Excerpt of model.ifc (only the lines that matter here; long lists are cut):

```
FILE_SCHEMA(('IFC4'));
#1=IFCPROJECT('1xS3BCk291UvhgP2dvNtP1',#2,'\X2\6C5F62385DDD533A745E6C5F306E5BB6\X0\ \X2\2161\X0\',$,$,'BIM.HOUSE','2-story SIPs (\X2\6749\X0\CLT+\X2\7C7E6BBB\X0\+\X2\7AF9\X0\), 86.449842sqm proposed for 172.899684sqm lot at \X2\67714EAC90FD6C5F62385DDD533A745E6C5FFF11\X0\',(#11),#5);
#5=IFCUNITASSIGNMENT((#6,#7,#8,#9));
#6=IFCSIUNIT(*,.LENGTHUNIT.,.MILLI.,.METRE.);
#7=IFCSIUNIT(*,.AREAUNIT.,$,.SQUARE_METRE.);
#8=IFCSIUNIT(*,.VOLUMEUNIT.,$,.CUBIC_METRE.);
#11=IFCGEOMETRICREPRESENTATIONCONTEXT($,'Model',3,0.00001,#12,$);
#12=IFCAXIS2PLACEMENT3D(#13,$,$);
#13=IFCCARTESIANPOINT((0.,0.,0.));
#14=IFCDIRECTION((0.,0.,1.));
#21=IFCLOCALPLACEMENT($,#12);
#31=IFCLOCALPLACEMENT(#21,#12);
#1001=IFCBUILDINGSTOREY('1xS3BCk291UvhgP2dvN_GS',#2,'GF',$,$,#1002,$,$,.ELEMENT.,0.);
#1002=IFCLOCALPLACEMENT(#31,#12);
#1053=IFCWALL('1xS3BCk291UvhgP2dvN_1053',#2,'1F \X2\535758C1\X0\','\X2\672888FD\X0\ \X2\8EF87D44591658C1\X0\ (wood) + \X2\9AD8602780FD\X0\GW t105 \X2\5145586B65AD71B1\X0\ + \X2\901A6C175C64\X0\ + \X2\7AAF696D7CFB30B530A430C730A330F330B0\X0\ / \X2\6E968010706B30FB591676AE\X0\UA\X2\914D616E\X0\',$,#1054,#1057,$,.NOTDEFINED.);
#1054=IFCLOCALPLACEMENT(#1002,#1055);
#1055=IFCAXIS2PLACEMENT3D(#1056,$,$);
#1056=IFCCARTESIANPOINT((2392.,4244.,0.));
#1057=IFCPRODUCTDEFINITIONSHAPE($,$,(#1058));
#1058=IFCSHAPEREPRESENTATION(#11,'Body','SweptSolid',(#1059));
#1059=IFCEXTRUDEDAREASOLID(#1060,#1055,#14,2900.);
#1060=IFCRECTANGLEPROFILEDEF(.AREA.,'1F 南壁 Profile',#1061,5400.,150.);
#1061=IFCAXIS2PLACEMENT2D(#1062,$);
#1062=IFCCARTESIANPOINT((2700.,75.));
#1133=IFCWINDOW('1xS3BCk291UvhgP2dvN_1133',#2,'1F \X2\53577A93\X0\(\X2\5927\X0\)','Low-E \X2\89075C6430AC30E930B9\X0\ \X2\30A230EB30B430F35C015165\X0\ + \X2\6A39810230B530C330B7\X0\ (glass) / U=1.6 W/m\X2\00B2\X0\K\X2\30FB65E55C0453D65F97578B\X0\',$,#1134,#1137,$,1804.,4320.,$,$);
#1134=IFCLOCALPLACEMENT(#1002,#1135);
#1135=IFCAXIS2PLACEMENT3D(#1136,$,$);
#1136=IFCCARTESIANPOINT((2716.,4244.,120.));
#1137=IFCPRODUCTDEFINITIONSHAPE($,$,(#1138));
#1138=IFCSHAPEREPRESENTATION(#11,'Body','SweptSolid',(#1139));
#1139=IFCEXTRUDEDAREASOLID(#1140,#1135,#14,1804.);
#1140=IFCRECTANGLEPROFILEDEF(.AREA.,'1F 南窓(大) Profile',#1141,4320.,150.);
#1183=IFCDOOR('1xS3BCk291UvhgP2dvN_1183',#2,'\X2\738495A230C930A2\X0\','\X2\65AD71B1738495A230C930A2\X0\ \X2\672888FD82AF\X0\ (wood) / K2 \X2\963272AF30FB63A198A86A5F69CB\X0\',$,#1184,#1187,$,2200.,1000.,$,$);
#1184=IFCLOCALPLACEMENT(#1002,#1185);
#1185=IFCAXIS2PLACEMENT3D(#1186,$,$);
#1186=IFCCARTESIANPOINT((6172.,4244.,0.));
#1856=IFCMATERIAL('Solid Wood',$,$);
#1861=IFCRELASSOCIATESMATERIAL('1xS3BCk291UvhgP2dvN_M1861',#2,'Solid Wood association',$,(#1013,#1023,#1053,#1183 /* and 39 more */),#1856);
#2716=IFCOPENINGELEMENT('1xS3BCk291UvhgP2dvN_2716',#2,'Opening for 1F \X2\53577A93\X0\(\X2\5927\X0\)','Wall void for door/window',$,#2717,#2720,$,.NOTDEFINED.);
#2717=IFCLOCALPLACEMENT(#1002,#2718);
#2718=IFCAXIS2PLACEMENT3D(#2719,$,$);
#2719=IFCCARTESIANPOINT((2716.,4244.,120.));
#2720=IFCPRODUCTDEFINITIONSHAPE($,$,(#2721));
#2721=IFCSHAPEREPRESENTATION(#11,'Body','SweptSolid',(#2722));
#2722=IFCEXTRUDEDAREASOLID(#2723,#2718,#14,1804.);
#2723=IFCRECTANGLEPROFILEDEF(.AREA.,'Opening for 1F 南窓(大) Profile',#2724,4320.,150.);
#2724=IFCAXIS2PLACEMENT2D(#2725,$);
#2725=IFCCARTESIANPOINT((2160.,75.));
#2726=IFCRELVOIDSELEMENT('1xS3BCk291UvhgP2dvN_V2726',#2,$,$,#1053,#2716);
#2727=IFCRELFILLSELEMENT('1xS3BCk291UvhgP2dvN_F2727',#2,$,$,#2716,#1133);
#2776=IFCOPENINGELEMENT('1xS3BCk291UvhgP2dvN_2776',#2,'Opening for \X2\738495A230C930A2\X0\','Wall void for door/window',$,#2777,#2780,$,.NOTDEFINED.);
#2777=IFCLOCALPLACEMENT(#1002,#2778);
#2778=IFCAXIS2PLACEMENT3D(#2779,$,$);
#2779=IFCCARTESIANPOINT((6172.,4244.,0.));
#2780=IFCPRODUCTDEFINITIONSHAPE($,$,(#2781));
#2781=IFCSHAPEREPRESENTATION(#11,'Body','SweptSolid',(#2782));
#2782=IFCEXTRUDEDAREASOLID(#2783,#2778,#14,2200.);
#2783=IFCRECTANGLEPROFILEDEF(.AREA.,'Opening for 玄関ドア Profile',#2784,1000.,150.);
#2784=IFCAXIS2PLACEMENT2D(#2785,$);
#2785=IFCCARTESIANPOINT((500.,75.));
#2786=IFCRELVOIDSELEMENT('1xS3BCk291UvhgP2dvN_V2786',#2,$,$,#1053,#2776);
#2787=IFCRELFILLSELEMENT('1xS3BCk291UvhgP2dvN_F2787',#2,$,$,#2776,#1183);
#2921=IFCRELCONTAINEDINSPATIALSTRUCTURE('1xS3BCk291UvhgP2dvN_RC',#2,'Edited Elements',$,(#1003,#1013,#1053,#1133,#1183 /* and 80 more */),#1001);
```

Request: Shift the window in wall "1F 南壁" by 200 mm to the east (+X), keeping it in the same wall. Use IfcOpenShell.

```python
import ifcopenshell
import ifcopenshell.api.geometry
import ifcopenshell.util.placement

model = ifcopenshell.open("model.ifc")

window = model.by_guid("1xS3BCk291UvhgP2dvN_1133")
opening = window.FillsVoids[0].RelatingOpeningElement
wall = opening.VoidsElements[0].RelatingBuildingElement

wall_matrix = ifcopenshell.util.placement.get_local_placement(wall.ObjectPlacement)
shift = wall_matrix[:3, 0] * 200.0
before = ifcopenshell.util.placement.get_local_placement(window.ObjectPlacement)[:3, 3].copy()

# The window is not placed relative to its opening, so move both.
for product in (opening, window):
    matrix = ifcopenshell.util.placement.get_local_placement(product.ObjectPlacement)
    matrix[:3, 3] += shift
    ifcopenshell.api.geometry.edit_object_placement(model, product=product, matrix=matrix, is_si=False)

after = ifcopenshell.util.placement.get_local_placement(window.ObjectPlacement)[:3, 3]
print("window moved by", (after - before).round(3) + 0.0)

model.write("model-out.ifc")
```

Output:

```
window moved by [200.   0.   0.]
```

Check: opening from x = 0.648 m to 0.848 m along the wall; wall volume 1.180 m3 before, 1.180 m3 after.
